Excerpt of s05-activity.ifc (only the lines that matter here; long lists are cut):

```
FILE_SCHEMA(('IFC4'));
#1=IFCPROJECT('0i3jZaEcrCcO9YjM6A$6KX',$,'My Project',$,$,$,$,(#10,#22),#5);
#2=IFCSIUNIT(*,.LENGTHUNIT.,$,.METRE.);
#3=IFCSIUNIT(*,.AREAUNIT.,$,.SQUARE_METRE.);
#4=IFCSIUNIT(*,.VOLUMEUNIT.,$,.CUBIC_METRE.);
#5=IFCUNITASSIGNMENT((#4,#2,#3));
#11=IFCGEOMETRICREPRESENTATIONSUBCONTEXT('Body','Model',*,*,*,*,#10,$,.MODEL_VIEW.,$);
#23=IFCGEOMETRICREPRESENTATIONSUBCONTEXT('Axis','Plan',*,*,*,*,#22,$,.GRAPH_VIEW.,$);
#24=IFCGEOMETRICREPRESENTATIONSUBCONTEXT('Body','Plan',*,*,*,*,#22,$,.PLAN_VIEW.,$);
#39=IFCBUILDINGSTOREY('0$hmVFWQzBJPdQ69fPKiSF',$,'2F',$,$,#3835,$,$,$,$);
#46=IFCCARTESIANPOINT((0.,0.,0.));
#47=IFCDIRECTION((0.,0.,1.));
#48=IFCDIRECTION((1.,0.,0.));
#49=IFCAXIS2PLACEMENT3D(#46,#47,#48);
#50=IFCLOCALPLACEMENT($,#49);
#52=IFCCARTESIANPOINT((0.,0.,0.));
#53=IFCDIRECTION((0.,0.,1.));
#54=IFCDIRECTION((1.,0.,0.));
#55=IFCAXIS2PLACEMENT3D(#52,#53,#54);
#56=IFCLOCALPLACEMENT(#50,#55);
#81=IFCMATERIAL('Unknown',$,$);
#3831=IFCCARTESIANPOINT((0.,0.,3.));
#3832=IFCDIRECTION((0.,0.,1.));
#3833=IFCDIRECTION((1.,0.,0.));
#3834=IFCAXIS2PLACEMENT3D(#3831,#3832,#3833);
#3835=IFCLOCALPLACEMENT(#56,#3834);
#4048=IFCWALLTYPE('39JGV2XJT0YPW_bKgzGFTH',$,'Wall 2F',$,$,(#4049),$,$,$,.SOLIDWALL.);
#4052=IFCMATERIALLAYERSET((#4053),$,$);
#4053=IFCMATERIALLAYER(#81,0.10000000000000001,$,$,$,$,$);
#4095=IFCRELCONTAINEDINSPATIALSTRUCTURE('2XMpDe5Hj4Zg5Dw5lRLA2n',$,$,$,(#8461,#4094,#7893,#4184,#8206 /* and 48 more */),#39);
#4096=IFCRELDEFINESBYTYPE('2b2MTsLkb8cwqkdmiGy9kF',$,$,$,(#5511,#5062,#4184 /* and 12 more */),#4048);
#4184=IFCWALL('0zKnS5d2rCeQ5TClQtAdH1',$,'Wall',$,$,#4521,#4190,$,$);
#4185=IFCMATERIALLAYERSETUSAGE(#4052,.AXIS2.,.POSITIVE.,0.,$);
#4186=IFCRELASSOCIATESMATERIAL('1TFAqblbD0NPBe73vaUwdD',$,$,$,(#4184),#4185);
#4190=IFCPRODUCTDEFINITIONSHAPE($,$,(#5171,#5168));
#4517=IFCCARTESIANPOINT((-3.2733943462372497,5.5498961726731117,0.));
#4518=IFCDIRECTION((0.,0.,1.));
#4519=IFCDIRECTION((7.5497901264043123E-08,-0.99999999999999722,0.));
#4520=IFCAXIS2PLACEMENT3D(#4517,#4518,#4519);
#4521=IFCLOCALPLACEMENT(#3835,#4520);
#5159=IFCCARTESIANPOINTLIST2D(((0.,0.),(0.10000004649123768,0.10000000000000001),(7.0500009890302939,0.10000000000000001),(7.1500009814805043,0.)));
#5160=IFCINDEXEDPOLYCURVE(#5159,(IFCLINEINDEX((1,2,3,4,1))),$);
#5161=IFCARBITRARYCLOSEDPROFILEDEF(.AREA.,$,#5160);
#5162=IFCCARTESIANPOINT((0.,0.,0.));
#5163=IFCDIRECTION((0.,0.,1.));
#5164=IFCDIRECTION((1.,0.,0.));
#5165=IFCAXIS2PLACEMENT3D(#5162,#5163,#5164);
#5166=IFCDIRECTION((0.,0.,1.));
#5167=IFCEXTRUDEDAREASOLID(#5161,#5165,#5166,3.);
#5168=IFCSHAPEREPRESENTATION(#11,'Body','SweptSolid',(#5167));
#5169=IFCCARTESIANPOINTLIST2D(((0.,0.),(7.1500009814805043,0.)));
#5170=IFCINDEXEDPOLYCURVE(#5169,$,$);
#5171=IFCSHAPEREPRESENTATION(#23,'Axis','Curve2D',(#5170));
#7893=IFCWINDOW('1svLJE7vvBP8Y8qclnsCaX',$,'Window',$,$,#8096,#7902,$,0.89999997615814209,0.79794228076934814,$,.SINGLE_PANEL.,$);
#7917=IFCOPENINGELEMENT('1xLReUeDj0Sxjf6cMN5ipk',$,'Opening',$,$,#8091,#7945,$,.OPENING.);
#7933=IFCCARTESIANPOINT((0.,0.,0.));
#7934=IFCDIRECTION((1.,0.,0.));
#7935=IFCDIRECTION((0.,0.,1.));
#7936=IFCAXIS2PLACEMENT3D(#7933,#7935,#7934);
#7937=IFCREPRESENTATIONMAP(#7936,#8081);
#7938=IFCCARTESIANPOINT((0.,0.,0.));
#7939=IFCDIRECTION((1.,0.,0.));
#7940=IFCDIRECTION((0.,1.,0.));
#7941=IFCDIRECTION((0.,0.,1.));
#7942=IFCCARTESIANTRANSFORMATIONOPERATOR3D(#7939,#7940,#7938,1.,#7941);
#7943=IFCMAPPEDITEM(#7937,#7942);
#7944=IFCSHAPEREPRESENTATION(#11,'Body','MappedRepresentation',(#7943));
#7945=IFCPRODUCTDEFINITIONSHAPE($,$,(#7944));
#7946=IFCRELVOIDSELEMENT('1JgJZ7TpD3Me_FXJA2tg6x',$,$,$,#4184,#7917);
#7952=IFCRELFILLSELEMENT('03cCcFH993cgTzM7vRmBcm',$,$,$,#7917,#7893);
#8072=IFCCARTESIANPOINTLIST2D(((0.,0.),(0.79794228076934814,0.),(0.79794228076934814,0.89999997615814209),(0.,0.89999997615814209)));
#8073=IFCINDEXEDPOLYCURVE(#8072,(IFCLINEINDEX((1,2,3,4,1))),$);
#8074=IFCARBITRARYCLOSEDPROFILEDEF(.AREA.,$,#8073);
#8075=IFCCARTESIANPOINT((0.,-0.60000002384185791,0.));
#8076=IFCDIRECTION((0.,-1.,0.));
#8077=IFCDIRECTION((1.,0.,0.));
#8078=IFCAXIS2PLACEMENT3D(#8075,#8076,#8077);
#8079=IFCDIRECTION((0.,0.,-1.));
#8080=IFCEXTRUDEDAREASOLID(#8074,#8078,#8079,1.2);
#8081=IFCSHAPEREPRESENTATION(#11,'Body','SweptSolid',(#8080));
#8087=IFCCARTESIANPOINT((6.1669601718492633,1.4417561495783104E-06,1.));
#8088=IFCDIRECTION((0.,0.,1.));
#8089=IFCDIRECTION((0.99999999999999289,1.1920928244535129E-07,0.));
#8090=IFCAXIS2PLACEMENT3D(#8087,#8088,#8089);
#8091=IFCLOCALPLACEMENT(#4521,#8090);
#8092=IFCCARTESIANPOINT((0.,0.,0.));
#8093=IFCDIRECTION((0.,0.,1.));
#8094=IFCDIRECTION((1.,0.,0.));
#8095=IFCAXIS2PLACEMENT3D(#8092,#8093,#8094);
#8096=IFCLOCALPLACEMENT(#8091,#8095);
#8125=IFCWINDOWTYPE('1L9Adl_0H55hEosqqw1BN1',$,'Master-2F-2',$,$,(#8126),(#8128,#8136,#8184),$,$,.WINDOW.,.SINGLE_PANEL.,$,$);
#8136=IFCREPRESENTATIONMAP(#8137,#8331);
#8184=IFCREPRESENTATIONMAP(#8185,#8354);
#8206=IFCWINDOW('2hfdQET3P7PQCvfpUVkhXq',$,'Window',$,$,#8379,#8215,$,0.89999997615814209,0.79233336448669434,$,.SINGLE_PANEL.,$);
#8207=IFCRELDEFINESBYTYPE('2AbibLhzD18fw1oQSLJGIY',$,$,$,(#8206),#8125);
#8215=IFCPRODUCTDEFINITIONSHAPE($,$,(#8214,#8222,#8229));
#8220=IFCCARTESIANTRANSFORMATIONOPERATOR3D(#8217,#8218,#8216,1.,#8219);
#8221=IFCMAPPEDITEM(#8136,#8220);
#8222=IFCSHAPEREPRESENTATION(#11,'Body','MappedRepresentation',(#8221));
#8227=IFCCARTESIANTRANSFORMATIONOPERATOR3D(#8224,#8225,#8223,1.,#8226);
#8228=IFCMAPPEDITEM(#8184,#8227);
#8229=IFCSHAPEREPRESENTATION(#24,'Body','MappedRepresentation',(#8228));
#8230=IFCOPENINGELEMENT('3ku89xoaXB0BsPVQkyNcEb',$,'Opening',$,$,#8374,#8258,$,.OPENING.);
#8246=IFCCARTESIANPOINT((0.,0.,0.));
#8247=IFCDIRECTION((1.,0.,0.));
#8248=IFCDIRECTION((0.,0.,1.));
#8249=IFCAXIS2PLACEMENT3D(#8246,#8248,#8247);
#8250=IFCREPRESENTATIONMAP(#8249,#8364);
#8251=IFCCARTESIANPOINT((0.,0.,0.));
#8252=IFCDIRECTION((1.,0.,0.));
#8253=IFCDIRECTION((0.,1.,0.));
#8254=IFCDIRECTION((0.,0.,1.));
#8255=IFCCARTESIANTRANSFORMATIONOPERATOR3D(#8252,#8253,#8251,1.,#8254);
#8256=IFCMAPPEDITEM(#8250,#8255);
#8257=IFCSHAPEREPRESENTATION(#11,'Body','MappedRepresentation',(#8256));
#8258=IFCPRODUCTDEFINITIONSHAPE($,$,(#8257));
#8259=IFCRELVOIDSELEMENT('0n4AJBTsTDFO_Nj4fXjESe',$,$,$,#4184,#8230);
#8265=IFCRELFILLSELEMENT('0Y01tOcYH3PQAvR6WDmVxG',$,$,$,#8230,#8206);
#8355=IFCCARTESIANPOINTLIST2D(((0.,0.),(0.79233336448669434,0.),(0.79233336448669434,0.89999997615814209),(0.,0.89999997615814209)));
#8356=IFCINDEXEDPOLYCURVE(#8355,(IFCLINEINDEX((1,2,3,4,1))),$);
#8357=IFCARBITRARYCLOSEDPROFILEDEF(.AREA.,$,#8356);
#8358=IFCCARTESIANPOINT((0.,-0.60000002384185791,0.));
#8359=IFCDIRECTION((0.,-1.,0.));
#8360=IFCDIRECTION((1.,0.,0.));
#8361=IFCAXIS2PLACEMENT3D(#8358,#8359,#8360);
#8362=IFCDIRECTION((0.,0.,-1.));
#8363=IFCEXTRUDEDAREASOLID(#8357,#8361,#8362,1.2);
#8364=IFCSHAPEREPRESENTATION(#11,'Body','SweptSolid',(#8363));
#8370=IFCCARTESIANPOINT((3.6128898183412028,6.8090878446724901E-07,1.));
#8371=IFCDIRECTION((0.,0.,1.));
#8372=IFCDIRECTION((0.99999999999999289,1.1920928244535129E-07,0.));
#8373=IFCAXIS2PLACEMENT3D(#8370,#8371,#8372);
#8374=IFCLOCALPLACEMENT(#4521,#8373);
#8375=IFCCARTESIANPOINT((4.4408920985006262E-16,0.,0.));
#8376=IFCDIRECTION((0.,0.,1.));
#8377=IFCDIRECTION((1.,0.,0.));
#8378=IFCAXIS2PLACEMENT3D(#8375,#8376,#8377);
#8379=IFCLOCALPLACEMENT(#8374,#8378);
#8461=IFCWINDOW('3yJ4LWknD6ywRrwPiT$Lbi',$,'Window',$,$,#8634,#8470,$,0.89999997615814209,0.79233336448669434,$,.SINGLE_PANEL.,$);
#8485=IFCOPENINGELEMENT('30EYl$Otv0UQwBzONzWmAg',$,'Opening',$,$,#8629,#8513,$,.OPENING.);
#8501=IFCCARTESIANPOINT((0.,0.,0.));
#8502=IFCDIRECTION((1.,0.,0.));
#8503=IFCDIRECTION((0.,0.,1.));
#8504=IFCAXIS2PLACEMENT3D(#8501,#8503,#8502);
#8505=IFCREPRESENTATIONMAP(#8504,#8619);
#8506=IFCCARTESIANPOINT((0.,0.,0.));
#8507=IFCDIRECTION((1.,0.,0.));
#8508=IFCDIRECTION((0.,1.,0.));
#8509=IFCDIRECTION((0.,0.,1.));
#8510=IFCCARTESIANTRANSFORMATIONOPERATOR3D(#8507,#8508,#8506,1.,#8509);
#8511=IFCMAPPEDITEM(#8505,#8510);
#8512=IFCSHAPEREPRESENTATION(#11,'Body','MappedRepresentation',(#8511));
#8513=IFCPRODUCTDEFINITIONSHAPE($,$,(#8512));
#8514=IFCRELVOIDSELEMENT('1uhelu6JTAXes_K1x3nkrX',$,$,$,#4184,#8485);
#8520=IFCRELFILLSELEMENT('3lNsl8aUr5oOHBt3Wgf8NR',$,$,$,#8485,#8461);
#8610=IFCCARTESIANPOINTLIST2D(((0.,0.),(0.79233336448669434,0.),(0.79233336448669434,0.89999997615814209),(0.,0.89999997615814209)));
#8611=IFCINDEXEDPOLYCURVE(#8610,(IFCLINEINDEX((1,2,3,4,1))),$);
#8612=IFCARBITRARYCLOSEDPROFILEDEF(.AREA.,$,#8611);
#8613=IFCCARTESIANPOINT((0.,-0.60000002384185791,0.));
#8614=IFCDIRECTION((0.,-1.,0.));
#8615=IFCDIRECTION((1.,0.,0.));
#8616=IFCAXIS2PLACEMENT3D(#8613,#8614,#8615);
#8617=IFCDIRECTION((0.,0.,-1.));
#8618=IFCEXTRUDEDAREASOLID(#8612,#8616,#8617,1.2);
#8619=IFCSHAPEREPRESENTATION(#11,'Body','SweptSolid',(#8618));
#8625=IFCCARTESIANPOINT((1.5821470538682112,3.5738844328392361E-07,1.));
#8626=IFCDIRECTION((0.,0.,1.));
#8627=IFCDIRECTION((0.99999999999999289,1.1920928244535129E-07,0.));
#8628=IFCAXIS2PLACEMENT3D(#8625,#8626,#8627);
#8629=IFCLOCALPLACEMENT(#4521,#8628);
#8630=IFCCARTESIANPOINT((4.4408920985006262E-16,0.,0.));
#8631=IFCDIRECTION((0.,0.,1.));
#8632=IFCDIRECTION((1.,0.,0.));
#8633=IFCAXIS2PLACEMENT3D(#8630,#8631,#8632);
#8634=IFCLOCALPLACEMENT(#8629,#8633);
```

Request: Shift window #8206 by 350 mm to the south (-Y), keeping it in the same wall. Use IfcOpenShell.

```python
import ifcopenshell
import ifcopenshell.api.geometry
import ifcopenshell.util.placement
import ifcopenshell.util.unit

model = ifcopenshell.open("s05-activity.ifc")
unit_scale = ifcopenshell.util.unit.calculate_unit_scale(model)

window = model.by_guid("2hfdQET3P7PQCvfpUVkhXq")
opening = window.FillsVoids[0].RelatingOpeningElement
wall = opening.VoidsElements[0].RelatingBuildingElement

wall_matrix = ifcopenshell.util.placement.get_local_placement(wall.ObjectPlacement)
shift = wall_matrix[:3, 0] * 0.35 / unit_scale
before = ifcopenshell.util.placement.get_local_placement(window.ObjectPlacement)[:3, 3].copy()

# The window is placed relative to its opening, so it follows when the opening moves.
matrix = ifcopenshell.util.placement.get_local_placement(opening.ObjectPlacement)
matrix[:3, 3] += shift
ifcopenshell.api.geometry.edit_object_placement(
    model, product=opening, matrix=matrix, is_si=False, should_transform_children=True
)

after = ifcopenshell.util.placement.get_local_placement(window.ObjectPlacement)[:3, 3]
print("window moved by", (after - before).round(3) + 0.0)

model.write("s05-activity_updated.ifc")
```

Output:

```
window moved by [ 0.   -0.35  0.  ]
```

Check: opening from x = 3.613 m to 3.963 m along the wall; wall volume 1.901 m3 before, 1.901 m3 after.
